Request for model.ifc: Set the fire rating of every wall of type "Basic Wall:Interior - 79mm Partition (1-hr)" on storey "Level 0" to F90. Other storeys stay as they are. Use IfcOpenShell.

First a look at what the model holds.

```python
import ifcopenshell
import ifcopenshell.util.element

model = ifcopenshell.open("model.ifc")
print(model.schema)
storey = next(s for s in model.by_type("IfcBuildingStorey") if s.Name == "Level 0")
walls = [e for e in ifcopenshell.util.element.get_decomposition(storey) if e.is_a("IfcWall")]
seen = {}
for e in walls:
    element_type = ifcopenshell.util.element.get_type(e)
    key = (element_type.Name if element_type != e and element_type else None, ifcopenshell.util.element.get_pset(e, "Pset_WallCommon", "FireRating"))
    seen[key] = seen.get(key, 0) + 1
for (name, value), count in sorted(seen.items(), key=str):
    print(count, "x", name, "|", value)
```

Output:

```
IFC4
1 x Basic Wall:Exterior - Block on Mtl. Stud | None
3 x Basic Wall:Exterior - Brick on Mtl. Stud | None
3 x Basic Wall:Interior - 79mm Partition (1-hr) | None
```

```python
import ifcopenshell
import ifcopenshell.api.pset
import ifcopenshell.util.element

model = ifcopenshell.open("model.ifc")

storey = next(s for s in model.by_type("IfcBuildingStorey") if s.Name == "Level 0")
walls = [e for e in ifcopenshell.util.element.get_decomposition(storey) if e.is_a("IfcWall")]

count = 0
for e in walls:
    element_type = ifcopenshell.util.element.get_type(e)
    if element_type in (None, e) or element_type.Name != "Basic Wall:Interior - 79mm Partition (1-hr)":
        continue
    # add_pset returns the element's existing set when there is one.
    pset = ifcopenshell.api.pset.add_pset(model, product=e, name="Pset_WallCommon")
    ifcopenshell.api.pset.edit_pset(model, pset=pset, properties={"FireRating": "F90"})
    count += 1

print(count, "walls updated")

model.write("model_updated.ifc")
```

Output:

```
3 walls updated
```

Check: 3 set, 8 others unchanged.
